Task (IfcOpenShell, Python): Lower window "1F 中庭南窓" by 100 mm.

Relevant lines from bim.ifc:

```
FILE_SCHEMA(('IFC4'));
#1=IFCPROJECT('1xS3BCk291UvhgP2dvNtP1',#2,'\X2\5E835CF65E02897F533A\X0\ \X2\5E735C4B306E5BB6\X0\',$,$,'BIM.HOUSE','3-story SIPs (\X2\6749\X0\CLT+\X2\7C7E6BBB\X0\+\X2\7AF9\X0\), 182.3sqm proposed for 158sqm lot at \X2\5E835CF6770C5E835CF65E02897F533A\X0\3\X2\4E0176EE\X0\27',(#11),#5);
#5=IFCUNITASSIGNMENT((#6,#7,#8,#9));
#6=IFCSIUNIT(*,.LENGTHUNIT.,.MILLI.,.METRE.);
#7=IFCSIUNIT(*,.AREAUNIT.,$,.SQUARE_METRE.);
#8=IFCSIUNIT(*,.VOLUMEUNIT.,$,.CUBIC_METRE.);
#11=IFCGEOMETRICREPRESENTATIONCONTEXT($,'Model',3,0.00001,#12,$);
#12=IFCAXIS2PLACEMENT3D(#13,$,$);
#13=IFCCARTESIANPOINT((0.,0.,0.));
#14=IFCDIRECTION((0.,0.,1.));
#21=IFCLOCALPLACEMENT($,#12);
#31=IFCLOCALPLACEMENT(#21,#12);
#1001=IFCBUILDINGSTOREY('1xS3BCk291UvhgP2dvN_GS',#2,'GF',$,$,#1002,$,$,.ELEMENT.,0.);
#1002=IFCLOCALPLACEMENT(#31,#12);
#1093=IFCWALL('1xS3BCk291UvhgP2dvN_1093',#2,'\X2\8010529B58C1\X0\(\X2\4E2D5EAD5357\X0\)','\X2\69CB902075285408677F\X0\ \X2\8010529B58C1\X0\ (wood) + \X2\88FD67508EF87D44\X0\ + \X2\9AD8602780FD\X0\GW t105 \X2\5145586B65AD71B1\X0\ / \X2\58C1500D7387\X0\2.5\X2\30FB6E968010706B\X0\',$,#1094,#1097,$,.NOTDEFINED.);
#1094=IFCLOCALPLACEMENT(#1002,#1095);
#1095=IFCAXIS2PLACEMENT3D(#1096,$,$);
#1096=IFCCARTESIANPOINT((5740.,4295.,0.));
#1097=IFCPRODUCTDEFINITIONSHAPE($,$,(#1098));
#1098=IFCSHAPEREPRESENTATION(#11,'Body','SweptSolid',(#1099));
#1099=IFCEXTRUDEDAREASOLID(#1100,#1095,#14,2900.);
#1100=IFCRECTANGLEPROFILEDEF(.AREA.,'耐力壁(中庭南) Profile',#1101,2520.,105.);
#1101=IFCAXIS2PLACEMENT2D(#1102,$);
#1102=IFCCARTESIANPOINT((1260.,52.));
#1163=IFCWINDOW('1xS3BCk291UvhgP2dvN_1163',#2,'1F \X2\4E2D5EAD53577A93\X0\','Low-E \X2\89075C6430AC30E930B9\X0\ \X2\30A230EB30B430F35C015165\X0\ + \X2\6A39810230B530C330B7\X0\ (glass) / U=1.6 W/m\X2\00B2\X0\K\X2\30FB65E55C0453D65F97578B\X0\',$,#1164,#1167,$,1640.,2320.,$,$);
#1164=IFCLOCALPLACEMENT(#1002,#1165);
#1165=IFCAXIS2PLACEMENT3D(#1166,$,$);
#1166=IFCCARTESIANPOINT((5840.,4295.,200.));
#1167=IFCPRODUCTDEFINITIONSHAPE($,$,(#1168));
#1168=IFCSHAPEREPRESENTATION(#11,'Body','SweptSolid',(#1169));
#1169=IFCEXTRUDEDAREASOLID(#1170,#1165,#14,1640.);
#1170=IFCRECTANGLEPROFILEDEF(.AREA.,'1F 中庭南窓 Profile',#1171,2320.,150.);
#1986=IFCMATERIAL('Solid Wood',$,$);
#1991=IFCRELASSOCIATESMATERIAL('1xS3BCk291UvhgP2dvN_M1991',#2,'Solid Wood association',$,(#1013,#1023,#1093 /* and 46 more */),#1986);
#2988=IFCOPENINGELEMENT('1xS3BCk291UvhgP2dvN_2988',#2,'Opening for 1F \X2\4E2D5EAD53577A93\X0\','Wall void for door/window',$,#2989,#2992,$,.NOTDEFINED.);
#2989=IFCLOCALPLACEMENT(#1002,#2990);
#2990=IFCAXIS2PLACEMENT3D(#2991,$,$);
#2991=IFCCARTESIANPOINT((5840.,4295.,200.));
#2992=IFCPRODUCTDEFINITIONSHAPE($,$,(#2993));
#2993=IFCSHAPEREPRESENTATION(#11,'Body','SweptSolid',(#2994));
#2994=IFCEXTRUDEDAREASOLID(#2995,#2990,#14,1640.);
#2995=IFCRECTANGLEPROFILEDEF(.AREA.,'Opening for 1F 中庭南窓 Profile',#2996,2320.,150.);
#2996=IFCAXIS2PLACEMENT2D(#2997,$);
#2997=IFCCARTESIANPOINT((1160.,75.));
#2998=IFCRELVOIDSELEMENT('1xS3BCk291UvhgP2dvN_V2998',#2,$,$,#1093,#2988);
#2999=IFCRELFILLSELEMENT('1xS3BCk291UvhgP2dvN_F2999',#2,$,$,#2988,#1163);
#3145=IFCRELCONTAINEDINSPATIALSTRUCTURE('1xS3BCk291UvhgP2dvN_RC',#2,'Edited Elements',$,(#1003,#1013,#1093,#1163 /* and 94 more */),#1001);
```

```python
import numpy as np
import ifcopenshell
import ifcopenshell.api.geometry
import ifcopenshell.util.placement
import ifcopenshell.util.unit

model = ifcopenshell.open("bim.ifc")
unit_scale = ifcopenshell.util.unit.calculate_unit_scale(model)

window = model.by_guid("1xS3BCk291UvhgP2dvN_1163")
opening = window.FillsVoids[0].RelatingOpeningElement
dz = -100.0

shift = np.array([0.0, 0.0, dz])
# The window is not placed relative to its opening, so move both.
for product in (opening, window):
    matrix = ifcopenshell.util.placement.get_local_placement(product.ObjectPlacement)
    matrix[:3, 3] += shift
    ifcopenshell.api.geometry.edit_object_placement(model, product=product, matrix=matrix, is_si=False)

print(f"moved by {dz * unit_scale:+.3f} m")

model.write("bim-out.ifc")
```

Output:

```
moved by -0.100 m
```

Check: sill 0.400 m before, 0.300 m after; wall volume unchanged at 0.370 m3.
